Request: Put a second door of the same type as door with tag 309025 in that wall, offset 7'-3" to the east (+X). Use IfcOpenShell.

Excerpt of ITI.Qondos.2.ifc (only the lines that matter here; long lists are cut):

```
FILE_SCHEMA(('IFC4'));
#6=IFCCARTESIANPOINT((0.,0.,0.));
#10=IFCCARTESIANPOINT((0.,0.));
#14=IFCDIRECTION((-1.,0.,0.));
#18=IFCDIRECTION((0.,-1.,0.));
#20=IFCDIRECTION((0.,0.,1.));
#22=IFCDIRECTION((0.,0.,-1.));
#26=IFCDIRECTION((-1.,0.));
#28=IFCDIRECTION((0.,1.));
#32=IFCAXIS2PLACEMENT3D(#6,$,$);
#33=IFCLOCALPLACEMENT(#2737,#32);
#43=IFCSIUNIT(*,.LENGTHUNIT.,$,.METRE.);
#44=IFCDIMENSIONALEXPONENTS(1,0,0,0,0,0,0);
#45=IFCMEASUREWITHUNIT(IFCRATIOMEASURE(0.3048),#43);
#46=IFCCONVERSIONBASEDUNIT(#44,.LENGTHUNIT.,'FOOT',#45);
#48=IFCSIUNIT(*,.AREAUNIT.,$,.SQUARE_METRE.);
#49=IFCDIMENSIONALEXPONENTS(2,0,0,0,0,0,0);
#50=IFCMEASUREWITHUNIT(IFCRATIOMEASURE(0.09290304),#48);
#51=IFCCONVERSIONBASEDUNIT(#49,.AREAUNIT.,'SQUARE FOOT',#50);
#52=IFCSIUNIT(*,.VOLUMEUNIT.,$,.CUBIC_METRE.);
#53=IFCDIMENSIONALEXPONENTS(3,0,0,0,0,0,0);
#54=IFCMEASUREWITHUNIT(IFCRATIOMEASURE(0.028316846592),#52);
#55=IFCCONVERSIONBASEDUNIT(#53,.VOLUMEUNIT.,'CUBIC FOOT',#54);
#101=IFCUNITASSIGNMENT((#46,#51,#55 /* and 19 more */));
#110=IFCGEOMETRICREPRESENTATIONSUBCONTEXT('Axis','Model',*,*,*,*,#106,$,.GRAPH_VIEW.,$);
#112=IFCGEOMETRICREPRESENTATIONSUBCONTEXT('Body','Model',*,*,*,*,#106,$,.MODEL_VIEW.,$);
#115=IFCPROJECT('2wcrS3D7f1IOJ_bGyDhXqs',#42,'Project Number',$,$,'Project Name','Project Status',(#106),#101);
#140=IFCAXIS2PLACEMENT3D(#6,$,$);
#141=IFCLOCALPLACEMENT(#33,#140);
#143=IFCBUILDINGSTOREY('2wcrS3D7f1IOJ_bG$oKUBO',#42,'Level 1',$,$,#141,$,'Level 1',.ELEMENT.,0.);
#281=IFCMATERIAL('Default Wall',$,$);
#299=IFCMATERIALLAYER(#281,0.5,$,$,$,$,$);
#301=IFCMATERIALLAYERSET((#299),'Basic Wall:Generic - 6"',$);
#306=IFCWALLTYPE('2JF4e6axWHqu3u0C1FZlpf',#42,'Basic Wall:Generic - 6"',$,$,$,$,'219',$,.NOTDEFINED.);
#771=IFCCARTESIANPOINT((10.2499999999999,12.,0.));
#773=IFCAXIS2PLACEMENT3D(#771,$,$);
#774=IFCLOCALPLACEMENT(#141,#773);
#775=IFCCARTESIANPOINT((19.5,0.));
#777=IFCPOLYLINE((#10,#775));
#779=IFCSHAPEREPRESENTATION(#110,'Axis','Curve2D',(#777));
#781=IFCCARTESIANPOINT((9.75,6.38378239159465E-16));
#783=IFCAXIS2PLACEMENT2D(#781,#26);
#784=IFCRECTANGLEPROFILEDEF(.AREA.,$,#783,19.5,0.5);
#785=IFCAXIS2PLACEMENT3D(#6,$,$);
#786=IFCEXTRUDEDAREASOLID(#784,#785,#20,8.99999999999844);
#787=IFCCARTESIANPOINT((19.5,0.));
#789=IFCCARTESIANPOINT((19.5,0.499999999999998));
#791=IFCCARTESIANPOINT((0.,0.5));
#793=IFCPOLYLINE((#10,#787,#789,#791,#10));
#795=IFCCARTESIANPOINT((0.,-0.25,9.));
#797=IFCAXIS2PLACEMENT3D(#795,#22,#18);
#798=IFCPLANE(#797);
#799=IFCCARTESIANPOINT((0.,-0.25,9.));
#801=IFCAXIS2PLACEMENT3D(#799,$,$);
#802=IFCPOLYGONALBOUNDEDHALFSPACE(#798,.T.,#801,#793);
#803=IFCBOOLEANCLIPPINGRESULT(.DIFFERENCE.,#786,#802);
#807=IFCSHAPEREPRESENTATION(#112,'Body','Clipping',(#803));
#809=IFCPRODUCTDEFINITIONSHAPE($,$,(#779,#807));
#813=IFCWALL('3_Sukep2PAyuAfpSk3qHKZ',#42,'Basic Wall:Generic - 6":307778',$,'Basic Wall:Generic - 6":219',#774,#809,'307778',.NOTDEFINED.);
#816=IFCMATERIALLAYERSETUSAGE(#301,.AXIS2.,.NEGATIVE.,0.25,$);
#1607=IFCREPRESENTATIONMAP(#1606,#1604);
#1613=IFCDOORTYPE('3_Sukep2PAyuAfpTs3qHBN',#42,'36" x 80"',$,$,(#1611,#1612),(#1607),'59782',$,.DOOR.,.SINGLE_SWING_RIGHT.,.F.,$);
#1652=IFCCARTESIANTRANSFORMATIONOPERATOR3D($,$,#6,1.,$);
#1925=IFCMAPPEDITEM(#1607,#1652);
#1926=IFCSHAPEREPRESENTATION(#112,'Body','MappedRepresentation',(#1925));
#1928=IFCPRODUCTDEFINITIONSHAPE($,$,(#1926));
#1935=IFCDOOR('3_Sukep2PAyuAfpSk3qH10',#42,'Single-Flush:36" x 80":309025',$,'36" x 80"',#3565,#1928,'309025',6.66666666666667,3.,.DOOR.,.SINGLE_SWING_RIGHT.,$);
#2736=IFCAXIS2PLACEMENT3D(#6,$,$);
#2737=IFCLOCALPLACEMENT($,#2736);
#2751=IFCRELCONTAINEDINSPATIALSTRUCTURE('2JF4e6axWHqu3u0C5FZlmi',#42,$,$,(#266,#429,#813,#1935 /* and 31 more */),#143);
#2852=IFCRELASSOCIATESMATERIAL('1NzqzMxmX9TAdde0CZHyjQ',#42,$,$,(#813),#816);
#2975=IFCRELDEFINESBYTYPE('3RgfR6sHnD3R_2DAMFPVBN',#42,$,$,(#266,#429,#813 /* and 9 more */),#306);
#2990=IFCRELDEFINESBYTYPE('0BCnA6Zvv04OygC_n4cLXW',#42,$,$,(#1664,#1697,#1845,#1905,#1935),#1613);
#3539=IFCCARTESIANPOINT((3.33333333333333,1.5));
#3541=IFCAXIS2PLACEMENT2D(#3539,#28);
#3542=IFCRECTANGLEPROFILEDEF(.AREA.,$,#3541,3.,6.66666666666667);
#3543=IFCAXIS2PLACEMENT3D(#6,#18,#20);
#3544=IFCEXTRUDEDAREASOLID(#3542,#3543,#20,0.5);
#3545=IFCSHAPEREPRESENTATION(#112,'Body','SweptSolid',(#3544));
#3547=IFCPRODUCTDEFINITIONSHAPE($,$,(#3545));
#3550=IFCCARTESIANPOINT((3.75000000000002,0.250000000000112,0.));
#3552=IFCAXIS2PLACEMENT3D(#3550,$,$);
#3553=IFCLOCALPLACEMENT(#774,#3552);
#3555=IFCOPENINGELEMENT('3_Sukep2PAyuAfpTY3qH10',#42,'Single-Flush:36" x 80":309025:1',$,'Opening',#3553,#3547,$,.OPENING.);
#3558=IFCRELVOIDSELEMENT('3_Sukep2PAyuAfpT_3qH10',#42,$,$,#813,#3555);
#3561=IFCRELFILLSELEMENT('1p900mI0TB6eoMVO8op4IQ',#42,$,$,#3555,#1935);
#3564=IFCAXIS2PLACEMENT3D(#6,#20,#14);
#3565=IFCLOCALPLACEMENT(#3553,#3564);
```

```python
import ifcopenshell
import ifcopenshell.api.feature
import ifcopenshell.api.geometry
import ifcopenshell.api.root
import ifcopenshell.geom
import ifcopenshell.util.element
import ifcopenshell.util.placement
import ifcopenshell.util.shape
import ifcopenshell.util.unit

model = ifcopenshell.open("ITI.Qondos.2.ifc")
unit_scale = ifcopenshell.util.unit.calculate_unit_scale(model)
settings = ifcopenshell.geom.settings()


def volume(element):
    """Net volume in cubic metres, openings subtracted."""
    shape = ifcopenshell.geom.create_shape(settings, element)
    return ifcopenshell.util.shape.get_volume(shape.geometry)


def reuse_history(source, copy):
    """copy_class also copies each property set's owner history, people and application; keep the originals."""
    for rel in copy.IsDefinedBy:
        if rel.is_a("IfcRelDefinesByProperties") and (history := rel.RelatingPropertyDefinition.OwnerHistory):
            rel.RelatingPropertyDefinition.OwnerHistory = source.OwnerHistory
            ifcopenshell.util.element.remove_deep2(model, history)


door = model.by_id(1935)
opening = door.FillsVoids[0].RelatingOpeningElement
wall = opening.VoidsElements[0].RelatingBuildingElement
before = volume(wall)
shift = ifcopenshell.util.placement.get_local_placement(wall.ObjectPlacement)[:3, 0] * 87 * 0.0254 / unit_scale

# copy_class copies the void relationship, type, container and properties, but no geometry.
new_opening = ifcopenshell.api.root.copy_class(model, product=opening)
new_opening.Representation = ifcopenshell.util.element.copy_deep(
    model, opening.Representation, exclude=["IfcGeometricRepresentationContext", "IfcRepresentationMap"]
)
new_opening.Name = 'Single-Flush:36" x 80"'
new_door = ifcopenshell.api.root.copy_class(model, product=door)
new_door.Representation = ifcopenshell.util.element.copy_deep(
    model, door.Representation, exclude=["IfcGeometricRepresentationContext", "IfcRepresentationMap"]
)
new_door.Name = 'Single-Flush:36" x 80"'
new_door.Tag = None
reuse_history(door, new_door)
ifcopenshell.api.feature.add_filling(model, opening=new_opening, element=new_door)

for old, new in ((opening, new_opening), (door, new_door)):
    matrix = ifcopenshell.util.placement.get_local_placement(old.ObjectPlacement)
    matrix[:3, 3] += shift
    ifcopenshell.api.geometry.edit_object_placement(model, product=new, matrix=matrix, is_si=False)

after = volume(wall)

print(f"wall volume {before:.3f} -> {after:.3f} m3")

model.write("ITI.Qondos.2-out.ifc")
```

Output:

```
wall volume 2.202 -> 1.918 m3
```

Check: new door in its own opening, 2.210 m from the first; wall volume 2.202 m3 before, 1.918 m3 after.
